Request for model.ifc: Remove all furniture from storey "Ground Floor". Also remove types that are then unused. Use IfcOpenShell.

First a look at what the model holds.

```python
import ifcopenshell
import ifcopenshell.util.element

model = ifcopenshell.open("model.ifc")
print(model.schema)
storey = next(s for s in model.by_type("IfcBuildingStorey") if s.Name == "Ground Floor")
furniture = [e for e in ifcopenshell.util.element.get_decomposition(storey) if e.is_a("IfcFurnishingElement")]
seen = {}
for e in furniture:
    element_type = ifcopenshell.util.element.get_type(e)
    name = element_type.Name if element_type not in (None, e) else None
    seen[name] = seen.get(name, 0) + 1
for name, count in sorted(seen.items(), key=str):
    print(count, "x", name)
```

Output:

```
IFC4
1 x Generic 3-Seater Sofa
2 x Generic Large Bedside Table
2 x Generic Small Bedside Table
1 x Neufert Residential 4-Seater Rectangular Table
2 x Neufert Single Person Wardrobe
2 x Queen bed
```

```python
import ifcopenshell
import ifcopenshell.api.root
import ifcopenshell.util.element

model = ifcopenshell.open("model.ifc")

storey = next(s for s in model.by_type("IfcBuildingStorey") if s.Name == "Ground Floor")
furniture = [e for e in ifcopenshell.util.element.get_decomposition(storey) if e.is_a("IfcFurnishingElement")]
types = {ifcopenshell.util.element.get_type(e) for e in furniture} - {None, *furniture}

for e in furniture:
    ifcopenshell.api.root.remove_product(model, product=e)
print(len(furniture), "removed")

unused = [t for t in types if not ifcopenshell.util.element.get_types(t)]
for t in unused:
    ifcopenshell.api.root.remove_product(model, product=t)
print(len(unused), "unused types removed")

model.write("model_updated.ifc")
```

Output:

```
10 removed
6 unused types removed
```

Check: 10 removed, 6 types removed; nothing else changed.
